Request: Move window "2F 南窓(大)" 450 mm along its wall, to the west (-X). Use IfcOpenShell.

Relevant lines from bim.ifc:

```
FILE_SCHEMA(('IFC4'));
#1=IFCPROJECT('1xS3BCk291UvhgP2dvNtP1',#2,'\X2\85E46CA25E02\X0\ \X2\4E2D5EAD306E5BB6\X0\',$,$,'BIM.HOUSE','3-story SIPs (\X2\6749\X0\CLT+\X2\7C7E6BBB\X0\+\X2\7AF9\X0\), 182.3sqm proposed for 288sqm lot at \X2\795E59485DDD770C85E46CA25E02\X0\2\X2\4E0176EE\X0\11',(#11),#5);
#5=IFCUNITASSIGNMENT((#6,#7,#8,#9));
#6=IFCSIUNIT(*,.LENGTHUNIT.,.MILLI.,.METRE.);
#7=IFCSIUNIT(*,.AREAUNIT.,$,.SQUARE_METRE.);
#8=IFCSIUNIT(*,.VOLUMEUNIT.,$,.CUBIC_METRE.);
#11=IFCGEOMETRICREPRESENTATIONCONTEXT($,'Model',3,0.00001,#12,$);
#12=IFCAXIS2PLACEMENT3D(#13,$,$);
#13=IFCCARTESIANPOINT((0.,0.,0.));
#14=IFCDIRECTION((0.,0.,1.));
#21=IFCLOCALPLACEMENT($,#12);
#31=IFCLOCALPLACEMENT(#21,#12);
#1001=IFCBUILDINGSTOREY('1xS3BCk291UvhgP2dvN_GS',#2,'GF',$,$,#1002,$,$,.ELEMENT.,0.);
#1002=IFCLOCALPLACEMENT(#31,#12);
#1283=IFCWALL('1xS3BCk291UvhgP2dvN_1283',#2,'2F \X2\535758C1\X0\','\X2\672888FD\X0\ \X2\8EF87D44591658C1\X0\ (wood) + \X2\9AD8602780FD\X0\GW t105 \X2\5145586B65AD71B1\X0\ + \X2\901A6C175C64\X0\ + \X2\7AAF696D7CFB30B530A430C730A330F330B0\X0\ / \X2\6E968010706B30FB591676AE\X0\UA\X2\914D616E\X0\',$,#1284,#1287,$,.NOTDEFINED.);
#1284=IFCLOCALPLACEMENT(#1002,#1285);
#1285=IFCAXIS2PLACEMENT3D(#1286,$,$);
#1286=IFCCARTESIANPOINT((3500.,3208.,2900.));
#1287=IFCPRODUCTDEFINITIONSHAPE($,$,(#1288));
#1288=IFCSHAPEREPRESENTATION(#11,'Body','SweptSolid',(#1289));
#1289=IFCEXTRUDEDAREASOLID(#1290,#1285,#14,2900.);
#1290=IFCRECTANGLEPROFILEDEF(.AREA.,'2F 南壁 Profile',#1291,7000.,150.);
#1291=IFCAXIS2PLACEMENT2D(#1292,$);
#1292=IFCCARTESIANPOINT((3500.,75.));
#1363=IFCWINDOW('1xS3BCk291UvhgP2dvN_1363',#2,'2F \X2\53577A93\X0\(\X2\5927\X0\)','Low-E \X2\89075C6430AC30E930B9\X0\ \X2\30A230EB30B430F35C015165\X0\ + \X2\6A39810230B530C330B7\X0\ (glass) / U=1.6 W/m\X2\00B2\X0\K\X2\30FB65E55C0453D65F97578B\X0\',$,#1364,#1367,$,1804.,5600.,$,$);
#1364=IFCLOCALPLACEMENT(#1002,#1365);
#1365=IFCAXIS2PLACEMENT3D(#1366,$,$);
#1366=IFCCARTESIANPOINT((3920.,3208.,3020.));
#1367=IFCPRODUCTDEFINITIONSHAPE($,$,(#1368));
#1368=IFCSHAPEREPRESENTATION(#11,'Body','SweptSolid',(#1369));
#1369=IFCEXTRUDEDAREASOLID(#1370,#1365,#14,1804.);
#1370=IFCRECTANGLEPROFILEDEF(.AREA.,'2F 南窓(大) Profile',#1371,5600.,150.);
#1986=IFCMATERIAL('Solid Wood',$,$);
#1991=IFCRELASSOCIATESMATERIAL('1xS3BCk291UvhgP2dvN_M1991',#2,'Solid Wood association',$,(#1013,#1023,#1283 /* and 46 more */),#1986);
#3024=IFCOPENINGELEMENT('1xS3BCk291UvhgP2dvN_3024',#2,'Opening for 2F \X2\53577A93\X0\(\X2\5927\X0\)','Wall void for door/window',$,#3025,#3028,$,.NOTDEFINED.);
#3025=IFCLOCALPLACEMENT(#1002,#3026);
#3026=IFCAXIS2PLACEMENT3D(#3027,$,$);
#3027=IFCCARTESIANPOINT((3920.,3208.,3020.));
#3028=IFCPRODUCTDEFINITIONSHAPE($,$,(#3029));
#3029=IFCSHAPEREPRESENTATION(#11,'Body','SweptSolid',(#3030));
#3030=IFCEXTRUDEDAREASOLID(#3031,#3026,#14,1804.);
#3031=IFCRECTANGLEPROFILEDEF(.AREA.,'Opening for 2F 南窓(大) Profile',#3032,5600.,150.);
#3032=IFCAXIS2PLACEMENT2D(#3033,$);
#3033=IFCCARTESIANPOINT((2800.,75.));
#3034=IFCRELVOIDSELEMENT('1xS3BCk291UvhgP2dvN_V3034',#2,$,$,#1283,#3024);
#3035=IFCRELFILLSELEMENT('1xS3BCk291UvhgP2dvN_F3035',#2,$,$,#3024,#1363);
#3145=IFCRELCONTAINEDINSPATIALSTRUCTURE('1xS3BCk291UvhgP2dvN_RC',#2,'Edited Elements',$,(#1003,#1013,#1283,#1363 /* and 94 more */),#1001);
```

```python
import ifcopenshell
import ifcopenshell.api.geometry
import ifcopenshell.util.placement
import ifcopenshell.util.unit

model = ifcopenshell.open("bim.ifc")
unit_scale = ifcopenshell.util.unit.calculate_unit_scale(model)

window = model.by_guid("1xS3BCk291UvhgP2dvN_1363")
opening = window.FillsVoids[0].RelatingOpeningElement
wall = opening.VoidsElements[0].RelatingBuildingElement

wall_matrix = ifcopenshell.util.placement.get_local_placement(wall.ObjectPlacement)
shift = wall_matrix[:3, 0] * -0.45 / unit_scale
before = ifcopenshell.util.placement.get_local_placement(window.ObjectPlacement)[:3, 3].copy()

# The window is not placed relative to its opening, so move both.
for product in (opening, window):
    matrix = ifcopenshell.util.placement.get_local_placement(product.ObjectPlacement)
    matrix[:3, 3] += shift
    ifcopenshell.api.geometry.edit_object_placement(model, product=product, matrix=matrix, is_si=False)

after = ifcopenshell.util.placement.get_local_placement(window.ObjectPlacement)[:3, 3]
print("window moved by", (after - before).round(3) + 0.0)

model.write("bim_edited.ifc")
```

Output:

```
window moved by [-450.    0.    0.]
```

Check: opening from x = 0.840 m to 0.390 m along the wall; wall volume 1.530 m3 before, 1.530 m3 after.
